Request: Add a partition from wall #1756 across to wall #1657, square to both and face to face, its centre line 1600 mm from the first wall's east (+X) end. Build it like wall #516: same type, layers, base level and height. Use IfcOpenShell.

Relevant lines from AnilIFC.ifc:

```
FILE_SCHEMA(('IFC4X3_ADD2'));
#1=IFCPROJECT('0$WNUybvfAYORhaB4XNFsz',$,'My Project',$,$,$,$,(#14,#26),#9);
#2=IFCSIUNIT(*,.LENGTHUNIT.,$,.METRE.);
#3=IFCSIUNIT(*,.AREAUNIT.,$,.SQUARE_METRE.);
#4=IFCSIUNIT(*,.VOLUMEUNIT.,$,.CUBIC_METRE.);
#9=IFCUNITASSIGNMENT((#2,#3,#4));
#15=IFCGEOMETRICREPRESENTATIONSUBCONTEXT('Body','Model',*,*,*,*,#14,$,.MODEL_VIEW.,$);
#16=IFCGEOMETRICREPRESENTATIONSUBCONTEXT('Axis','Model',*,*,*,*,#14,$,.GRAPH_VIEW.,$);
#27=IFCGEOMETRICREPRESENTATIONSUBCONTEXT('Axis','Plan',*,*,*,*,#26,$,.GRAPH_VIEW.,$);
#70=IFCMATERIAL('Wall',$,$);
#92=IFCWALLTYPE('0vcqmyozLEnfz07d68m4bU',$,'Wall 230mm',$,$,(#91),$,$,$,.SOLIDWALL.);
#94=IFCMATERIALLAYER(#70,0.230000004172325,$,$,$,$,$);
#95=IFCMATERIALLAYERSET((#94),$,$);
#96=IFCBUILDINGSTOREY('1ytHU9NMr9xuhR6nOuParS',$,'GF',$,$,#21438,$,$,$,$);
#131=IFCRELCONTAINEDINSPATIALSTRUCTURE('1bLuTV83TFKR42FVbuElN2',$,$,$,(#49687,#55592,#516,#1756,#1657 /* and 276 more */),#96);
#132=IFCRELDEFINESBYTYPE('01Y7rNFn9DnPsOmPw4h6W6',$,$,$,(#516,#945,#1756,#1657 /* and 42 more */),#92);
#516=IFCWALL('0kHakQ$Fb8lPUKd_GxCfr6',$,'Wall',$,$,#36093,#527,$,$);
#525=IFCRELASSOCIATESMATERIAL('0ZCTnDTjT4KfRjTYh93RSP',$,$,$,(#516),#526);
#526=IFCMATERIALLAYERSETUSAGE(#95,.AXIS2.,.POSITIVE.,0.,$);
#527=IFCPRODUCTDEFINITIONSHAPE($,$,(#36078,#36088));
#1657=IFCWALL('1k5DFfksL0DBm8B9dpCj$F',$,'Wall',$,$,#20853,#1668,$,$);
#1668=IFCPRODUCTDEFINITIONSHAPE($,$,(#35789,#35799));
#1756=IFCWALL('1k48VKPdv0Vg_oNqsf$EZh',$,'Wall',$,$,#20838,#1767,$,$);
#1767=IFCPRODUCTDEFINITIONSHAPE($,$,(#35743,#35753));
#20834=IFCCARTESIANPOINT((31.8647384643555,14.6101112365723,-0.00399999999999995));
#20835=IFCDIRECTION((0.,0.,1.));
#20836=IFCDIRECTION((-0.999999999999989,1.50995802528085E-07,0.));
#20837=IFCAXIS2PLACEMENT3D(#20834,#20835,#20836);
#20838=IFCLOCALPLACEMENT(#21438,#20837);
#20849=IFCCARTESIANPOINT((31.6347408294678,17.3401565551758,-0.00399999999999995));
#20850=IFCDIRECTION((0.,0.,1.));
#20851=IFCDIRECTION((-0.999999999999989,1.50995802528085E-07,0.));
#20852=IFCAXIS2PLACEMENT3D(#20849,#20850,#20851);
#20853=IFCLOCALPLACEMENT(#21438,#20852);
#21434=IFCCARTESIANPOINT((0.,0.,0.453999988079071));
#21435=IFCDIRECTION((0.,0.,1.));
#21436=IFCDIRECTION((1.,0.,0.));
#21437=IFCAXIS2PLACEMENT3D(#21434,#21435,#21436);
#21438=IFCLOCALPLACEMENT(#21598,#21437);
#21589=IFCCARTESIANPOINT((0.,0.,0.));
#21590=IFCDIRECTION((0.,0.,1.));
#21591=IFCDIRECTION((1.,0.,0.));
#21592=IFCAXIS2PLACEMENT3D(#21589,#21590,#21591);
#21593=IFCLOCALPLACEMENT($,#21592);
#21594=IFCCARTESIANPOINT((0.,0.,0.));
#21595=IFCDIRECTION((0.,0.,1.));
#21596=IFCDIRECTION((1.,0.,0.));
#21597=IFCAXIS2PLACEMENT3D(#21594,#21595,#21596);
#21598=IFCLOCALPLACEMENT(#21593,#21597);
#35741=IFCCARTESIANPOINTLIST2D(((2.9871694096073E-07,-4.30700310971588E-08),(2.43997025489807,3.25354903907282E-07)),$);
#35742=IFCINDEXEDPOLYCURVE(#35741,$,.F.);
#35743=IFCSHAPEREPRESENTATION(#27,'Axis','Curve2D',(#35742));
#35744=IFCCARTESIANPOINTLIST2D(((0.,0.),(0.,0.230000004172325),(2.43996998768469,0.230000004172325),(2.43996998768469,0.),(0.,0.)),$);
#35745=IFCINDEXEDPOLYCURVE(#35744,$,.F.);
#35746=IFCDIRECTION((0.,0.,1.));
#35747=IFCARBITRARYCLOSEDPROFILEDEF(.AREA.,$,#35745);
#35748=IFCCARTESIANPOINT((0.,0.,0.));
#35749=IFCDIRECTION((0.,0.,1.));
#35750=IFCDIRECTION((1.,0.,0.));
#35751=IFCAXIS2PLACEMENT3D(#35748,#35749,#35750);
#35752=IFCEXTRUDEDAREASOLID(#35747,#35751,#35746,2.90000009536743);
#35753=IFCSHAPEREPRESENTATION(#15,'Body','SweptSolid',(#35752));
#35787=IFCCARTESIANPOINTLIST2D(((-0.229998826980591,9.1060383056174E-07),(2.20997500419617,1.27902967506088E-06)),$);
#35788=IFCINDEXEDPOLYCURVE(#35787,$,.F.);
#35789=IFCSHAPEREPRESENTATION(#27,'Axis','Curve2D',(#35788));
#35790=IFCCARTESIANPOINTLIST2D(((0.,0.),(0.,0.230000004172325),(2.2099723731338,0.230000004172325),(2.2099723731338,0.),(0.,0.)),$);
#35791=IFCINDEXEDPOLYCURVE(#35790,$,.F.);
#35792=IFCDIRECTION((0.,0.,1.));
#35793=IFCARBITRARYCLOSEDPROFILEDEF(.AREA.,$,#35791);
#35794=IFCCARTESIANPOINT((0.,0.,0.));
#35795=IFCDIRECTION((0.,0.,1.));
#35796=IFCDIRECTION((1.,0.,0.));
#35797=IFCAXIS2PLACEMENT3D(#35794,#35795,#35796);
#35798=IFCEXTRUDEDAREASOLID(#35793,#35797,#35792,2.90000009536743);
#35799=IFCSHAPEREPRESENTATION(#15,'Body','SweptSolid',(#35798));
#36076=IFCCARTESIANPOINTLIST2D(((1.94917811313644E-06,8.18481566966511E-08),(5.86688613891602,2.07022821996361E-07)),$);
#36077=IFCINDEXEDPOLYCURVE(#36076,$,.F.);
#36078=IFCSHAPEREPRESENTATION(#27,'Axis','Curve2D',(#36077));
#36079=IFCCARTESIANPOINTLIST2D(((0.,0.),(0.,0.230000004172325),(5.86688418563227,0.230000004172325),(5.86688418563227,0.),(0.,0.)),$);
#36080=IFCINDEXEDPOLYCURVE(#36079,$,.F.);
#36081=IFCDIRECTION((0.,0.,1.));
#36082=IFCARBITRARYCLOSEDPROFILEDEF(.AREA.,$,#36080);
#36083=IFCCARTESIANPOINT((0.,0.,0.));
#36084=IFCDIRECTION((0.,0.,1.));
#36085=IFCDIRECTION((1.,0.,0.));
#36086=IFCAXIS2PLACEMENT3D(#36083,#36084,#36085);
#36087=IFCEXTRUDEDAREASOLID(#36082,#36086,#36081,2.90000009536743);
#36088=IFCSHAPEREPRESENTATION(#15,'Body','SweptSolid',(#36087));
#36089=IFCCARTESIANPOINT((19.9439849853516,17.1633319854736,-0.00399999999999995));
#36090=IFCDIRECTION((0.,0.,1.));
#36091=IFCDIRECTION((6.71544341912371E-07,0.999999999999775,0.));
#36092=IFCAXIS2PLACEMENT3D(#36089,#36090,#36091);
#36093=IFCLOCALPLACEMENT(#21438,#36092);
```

```python
import numpy as np
import ifcopenshell
import ifcopenshell.api.geometry
import ifcopenshell.api.material
import ifcopenshell.api.pset
import ifcopenshell.api.root
import ifcopenshell.api.spatial
import ifcopenshell.api.type
import ifcopenshell.geom
import ifcopenshell.util.element
import ifcopenshell.util.placement
import ifcopenshell.util.representation
import ifcopenshell.util.shape
import ifcopenshell.util.unit

model = ifcopenshell.open("AnilIFC.ifc")
unit_scale = ifcopenshell.util.unit.calculate_unit_scale(model)
settings = ifcopenshell.geom.settings()
settings.set("use-world-coords", True)

start_wall = model.by_guid("1k48VKPdv0Vg_oNqsf$EZh")
end_wall = model.by_id(1657)
like = model.by_guid("0kHakQ$Fb8lPUKd_GxCfr6")
matrix = ifcopenshell.util.placement.get_local_placement(start_wall.ObjectPlacement)
matrix[:3, 3] *= unit_scale


def extent(element):
    """Bounding box in the first wall's axes, in metres."""
    shape = ifcopenshell.geom.create_shape(settings, element)
    points = (ifcopenshell.util.shape.get_vertices(shape.geometry) - matrix[:3, 3]) @ matrix[:3, :3]
    return points.min(axis=0), points.max(axis=0)


y_start = extent(start_wall)[0][1]
y_end = extent(end_wall)[1][1]
like_min, like_max = extent(like)
length, height = float(abs(y_end - y_start)), float(like_max[2] - like_min[2])
layer_set = ifcopenshell.util.element.get_material(like, should_skip_usage=True)
thickness = sum(layer.LayerThickness for layer in layer_set.MaterialLayers) * unit_scale

wall = ifcopenshell.api.root.create_entity(model, ifc_class="IfcWall", name="New partition")
storey = ifcopenshell.util.element.get_container(like)
ifcopenshell.api.spatial.assign_container(model, products=[wall], relating_structure=storey)
ifcopenshell.api.type.assign_type(
    model, related_objects=[wall], relating_type=ifcopenshell.util.element.get_type(like), should_map_representations=False
)
rel = ifcopenshell.api.material.assign_material(
    model, products=[wall], type="IfcMaterialLayerSetUsage", material=layer_set
)
rel.RelatingMaterial.OffsetFromReferenceLine = -thickness / 2 / unit_scale
pset = ifcopenshell.api.pset.add_pset(model, product=wall, name="Pset_WallCommon")
ifcopenshell.api.pset.edit_pset(model, pset=pset, properties={"IsExternal": False, "LoadBearing": False})

# The axis runs down the middle of the wall.
axis = ifcopenshell.api.geometry.add_axis_representation(
    model, context=ifcopenshell.util.representation.get_context(model, "Model", "Axis"), axis=[(0.0, 0.0), (length, 0.0)]
)
body = ifcopenshell.api.geometry.add_wall_representation(
    model,
    context=ifcopenshell.util.representation.get_context(model, "Model", "Body", "MODEL_VIEW"),
    length=length,
    height=height,
    thickness=thickness,
    offset=-thickness / 2,
)
for representation in (axis, body):
    ifcopenshell.api.geometry.assign_representation(model, product=wall, representation=representation)

placement = matrix @ ifcopenshell.util.placement.rotation(-90, "Z")
placement[:, 3] = matrix @ np.array([extent(start_wall)[0][0] + 1.6, y_start, like_min[2], 1.0])
ifcopenshell.api.geometry.edit_object_placement(model, product=wall, matrix=placement)

print(f"partition {length:.3f} m long, {height:.3f} m high, {thickness:.3f} m thick")

model.write("AnilIFC_v2.ifc")
```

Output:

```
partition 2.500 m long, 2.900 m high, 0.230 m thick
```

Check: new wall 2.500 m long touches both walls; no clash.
